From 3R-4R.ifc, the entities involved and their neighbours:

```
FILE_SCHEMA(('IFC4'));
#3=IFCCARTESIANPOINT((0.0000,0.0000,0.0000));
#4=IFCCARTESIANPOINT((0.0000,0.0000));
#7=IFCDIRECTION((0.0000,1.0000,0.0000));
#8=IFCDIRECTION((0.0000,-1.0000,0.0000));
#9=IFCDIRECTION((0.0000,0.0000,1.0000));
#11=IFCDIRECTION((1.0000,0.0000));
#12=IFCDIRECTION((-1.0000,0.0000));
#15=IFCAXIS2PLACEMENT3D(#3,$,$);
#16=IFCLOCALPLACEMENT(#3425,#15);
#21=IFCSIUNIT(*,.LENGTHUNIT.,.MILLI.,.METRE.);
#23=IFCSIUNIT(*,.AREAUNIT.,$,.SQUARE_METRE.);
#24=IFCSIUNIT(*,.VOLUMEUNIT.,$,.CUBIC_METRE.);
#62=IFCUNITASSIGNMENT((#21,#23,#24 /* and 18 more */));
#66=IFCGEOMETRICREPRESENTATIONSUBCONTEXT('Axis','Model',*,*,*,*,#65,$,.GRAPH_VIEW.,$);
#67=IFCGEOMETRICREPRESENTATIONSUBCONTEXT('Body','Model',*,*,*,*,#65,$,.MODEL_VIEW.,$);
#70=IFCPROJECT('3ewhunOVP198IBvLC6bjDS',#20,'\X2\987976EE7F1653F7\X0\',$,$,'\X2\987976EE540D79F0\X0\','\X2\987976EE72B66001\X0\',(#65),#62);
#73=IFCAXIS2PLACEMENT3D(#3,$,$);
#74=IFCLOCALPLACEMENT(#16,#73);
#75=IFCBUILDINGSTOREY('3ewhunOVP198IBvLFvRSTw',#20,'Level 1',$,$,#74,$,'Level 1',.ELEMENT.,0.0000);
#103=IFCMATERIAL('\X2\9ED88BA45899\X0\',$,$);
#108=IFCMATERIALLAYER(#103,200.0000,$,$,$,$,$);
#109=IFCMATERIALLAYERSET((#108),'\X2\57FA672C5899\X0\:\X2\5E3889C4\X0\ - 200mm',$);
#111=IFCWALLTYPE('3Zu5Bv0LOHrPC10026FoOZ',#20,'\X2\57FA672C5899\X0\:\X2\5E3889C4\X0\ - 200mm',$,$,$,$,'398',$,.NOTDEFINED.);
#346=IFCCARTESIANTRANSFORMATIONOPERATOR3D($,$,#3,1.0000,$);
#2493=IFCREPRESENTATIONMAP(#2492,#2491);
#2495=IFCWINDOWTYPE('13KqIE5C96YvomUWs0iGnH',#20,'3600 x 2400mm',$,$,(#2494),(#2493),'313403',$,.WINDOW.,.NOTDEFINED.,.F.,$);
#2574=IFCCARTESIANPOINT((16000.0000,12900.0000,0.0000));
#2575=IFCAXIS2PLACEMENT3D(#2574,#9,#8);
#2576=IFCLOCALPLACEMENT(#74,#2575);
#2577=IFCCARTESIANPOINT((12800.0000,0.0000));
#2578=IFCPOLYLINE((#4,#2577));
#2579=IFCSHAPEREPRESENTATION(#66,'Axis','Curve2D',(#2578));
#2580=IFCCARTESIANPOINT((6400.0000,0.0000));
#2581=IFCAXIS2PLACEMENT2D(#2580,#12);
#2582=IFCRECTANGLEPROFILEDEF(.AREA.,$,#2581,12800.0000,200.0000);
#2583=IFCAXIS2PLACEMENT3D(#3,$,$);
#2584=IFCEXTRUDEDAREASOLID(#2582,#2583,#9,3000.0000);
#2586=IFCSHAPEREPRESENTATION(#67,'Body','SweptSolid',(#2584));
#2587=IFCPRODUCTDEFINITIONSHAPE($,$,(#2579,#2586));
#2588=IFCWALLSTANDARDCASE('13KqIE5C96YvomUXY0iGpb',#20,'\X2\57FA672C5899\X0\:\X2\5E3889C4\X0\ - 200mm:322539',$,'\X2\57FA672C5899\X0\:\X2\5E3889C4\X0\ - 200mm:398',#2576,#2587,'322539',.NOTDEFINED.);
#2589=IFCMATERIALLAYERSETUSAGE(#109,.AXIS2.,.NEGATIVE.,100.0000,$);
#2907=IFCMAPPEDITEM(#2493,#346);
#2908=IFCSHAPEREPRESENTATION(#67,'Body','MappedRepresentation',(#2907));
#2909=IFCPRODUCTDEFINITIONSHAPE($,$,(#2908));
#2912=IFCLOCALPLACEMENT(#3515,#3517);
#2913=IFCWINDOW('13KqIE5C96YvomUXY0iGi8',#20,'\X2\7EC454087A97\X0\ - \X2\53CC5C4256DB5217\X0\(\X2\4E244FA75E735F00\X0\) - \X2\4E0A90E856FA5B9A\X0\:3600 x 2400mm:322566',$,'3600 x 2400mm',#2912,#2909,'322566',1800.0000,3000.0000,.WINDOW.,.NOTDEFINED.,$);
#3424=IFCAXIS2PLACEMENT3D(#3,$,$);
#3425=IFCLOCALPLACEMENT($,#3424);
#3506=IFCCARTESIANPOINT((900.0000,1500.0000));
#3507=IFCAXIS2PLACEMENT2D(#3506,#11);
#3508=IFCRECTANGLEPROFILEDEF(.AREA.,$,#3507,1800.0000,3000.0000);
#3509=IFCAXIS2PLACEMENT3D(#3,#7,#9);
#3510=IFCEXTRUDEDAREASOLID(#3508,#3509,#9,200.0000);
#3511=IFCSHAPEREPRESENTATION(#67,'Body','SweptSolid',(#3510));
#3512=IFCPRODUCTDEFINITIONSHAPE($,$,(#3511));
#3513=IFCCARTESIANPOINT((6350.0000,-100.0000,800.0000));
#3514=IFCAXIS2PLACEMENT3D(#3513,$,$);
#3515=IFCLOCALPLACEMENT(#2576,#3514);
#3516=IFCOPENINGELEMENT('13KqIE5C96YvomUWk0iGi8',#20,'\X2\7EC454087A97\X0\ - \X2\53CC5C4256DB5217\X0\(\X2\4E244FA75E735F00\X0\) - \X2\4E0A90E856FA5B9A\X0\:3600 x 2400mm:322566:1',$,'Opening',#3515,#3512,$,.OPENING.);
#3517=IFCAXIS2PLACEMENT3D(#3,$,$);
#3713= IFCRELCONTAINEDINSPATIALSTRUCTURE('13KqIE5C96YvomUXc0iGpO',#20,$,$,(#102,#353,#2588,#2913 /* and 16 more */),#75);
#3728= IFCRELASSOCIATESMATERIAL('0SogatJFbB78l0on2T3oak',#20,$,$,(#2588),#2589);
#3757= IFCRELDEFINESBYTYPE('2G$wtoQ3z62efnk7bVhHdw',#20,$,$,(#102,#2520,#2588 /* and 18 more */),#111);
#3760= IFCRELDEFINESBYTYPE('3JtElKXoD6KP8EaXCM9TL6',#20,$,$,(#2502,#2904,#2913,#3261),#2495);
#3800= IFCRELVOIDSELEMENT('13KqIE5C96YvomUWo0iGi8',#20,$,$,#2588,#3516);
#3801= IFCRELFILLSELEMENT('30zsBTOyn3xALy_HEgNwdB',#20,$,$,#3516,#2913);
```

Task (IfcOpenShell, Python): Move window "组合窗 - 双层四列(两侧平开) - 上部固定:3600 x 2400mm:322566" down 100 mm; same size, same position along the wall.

```python
import numpy as np
import ifcopenshell
import ifcopenshell.api.geometry
import ifcopenshell.util.placement
import ifcopenshell.util.unit

model = ifcopenshell.open("3R-4R.ifc")
unit_scale = ifcopenshell.util.unit.calculate_unit_scale(model)

window = model.by_guid("13KqIE5C96YvomUXY0iGi8")
opening = window.FillsVoids[0].RelatingOpeningElement
dz = -100.0

shift = np.array([0.0, 0.0, dz])
# The window is placed relative to its opening, so it follows when the opening moves.
matrix = ifcopenshell.util.placement.get_local_placement(opening.ObjectPlacement)
matrix[:3, 3] += shift
ifcopenshell.api.geometry.edit_object_placement(
    model, product=opening, matrix=matrix, is_si=False, should_transform_children=True
)

print(f"moved by {dz * unit_scale:+.3f} m")

model.write("3R-4R_v2.ifc")
```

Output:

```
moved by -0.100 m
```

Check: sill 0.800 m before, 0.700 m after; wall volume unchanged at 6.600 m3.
